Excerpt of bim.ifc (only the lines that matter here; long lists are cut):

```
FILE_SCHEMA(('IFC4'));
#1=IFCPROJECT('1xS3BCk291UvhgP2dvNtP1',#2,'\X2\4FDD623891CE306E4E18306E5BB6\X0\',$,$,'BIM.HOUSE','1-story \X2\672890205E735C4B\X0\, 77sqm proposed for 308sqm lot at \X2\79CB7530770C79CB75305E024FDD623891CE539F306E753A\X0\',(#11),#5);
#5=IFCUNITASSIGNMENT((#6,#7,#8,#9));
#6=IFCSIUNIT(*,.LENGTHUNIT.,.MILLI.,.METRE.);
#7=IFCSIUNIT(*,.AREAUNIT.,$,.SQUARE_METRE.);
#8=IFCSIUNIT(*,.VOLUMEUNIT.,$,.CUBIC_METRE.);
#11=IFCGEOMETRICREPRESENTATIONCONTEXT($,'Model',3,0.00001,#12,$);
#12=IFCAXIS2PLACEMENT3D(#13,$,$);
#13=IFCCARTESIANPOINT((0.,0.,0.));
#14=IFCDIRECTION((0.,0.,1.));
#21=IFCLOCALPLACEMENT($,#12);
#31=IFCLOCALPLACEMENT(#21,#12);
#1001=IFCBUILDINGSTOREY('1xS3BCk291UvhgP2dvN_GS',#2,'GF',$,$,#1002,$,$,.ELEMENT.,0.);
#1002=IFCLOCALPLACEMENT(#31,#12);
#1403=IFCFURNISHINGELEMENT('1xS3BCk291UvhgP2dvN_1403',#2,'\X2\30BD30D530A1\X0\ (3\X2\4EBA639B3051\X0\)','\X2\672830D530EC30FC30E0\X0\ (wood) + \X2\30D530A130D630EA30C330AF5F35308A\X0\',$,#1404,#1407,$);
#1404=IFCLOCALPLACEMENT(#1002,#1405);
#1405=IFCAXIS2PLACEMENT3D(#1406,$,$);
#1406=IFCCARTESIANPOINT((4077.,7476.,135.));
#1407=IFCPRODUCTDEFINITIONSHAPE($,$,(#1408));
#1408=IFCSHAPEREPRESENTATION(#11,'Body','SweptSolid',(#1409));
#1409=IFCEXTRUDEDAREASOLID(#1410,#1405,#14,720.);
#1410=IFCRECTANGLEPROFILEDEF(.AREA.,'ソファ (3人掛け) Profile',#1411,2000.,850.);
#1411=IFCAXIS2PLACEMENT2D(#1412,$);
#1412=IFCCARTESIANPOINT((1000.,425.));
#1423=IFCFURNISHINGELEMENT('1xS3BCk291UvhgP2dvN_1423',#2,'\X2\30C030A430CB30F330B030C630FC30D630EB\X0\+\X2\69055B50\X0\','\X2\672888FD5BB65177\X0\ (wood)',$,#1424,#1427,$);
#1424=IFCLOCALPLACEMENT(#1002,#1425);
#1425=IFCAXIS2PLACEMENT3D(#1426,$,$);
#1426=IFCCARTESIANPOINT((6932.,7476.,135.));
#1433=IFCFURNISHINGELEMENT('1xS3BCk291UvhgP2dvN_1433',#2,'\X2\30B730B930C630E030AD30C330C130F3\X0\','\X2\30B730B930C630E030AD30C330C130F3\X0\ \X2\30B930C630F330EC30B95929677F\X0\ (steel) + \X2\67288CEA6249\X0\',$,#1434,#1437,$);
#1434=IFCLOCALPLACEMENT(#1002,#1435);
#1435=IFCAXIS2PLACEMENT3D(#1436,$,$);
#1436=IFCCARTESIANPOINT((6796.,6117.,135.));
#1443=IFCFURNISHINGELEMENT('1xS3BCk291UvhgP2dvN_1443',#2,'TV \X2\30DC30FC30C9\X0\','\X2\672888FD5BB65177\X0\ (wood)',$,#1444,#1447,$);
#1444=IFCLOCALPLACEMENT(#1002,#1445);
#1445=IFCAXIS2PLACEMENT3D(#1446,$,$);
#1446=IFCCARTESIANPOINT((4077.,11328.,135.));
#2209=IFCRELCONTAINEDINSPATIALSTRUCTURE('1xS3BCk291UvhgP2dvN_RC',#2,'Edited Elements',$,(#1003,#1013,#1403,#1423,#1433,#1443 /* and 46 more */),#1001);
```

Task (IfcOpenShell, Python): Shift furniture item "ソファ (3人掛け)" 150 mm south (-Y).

```python
import ifcopenshell
import ifcopenshell.api.geometry
import ifcopenshell.util.placement
import ifcopenshell.util.unit

model = ifcopenshell.open("bim.ifc")
unit_scale = ifcopenshell.util.unit.calculate_unit_scale(model)

item = model.by_id(1403)
matrix = ifcopenshell.util.placement.get_local_placement(item.ObjectPlacement)
matrix[1, 3] -= 0.15 / unit_scale
ifcopenshell.api.geometry.edit_object_placement(model, product=item, matrix=matrix, is_si=False)

print(ifcopenshell.util.placement.get_local_placement(item.ObjectPlacement).round(3) + 0.0)

model.write("bim-out.ifc")
```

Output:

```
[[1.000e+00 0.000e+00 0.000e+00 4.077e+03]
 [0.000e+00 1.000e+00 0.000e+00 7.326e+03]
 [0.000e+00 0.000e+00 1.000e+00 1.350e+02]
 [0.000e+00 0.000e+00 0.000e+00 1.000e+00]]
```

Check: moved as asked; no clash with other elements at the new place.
